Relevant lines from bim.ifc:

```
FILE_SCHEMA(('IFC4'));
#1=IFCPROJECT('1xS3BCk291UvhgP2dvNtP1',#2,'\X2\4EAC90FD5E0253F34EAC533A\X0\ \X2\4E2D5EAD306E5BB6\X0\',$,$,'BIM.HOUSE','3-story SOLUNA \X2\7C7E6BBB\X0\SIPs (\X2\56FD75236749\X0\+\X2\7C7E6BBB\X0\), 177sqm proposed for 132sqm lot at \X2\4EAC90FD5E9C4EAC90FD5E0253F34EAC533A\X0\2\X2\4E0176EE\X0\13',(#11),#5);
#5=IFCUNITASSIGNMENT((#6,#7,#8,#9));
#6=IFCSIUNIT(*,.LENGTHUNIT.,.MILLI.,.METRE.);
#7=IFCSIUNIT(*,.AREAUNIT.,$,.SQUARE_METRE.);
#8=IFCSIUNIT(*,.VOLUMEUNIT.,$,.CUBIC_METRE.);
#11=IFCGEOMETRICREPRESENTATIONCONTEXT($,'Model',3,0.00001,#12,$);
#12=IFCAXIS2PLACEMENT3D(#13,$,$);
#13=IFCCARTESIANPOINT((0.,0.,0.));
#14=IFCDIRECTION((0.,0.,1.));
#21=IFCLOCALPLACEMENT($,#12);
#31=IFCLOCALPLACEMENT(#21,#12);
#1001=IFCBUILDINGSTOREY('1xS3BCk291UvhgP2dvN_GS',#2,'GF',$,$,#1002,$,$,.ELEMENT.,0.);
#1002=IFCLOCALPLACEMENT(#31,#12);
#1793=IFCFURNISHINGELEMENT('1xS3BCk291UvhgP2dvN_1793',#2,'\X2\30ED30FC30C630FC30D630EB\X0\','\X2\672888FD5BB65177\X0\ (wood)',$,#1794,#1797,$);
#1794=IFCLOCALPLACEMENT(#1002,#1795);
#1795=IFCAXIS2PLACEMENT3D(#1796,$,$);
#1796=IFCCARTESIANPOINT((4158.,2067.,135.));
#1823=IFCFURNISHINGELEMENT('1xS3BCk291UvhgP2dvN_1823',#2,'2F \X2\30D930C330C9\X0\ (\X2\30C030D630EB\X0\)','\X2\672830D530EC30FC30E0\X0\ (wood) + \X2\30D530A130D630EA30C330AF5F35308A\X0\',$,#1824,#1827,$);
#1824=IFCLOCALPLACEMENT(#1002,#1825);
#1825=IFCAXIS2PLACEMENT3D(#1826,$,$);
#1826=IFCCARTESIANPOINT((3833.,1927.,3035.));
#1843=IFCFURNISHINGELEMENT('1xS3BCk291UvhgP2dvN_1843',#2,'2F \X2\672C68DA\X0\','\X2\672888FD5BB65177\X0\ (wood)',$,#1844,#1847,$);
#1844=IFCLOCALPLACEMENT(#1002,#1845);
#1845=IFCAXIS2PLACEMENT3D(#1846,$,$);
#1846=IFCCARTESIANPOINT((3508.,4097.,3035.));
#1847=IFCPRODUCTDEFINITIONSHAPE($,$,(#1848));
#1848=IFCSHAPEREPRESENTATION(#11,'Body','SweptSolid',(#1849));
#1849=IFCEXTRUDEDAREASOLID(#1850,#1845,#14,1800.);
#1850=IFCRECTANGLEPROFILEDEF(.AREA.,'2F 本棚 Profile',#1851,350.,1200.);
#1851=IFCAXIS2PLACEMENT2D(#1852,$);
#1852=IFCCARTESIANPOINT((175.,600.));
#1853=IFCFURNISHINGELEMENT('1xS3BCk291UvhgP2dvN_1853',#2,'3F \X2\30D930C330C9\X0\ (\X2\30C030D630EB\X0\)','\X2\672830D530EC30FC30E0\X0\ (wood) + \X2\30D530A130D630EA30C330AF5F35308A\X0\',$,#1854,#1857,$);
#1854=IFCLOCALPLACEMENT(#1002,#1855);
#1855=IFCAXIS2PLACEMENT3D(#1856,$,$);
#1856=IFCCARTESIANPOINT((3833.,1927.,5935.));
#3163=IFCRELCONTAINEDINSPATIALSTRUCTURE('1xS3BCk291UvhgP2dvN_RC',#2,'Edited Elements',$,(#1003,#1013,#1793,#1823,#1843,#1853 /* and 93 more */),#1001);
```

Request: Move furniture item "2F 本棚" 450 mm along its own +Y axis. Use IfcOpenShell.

```python
import ifcopenshell
import ifcopenshell.api.geometry
import ifcopenshell.util.placement

model = ifcopenshell.open("bim.ifc")

item = model.by_id(1843)
matrix = ifcopenshell.util.placement.get_local_placement(item.ObjectPlacement)
matrix[:3, 3] += matrix[:3, 1] * 450.0
ifcopenshell.api.geometry.edit_object_placement(model, product=item, matrix=matrix, is_si=False)

print(ifcopenshell.util.placement.get_local_placement(item.ObjectPlacement).round(3) + 0.0)

model.write("bim_edited.ifc")
```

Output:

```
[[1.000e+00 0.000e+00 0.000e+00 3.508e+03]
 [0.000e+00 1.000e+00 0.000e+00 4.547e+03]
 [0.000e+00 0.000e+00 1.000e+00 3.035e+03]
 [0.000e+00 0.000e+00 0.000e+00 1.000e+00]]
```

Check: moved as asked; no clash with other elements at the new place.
